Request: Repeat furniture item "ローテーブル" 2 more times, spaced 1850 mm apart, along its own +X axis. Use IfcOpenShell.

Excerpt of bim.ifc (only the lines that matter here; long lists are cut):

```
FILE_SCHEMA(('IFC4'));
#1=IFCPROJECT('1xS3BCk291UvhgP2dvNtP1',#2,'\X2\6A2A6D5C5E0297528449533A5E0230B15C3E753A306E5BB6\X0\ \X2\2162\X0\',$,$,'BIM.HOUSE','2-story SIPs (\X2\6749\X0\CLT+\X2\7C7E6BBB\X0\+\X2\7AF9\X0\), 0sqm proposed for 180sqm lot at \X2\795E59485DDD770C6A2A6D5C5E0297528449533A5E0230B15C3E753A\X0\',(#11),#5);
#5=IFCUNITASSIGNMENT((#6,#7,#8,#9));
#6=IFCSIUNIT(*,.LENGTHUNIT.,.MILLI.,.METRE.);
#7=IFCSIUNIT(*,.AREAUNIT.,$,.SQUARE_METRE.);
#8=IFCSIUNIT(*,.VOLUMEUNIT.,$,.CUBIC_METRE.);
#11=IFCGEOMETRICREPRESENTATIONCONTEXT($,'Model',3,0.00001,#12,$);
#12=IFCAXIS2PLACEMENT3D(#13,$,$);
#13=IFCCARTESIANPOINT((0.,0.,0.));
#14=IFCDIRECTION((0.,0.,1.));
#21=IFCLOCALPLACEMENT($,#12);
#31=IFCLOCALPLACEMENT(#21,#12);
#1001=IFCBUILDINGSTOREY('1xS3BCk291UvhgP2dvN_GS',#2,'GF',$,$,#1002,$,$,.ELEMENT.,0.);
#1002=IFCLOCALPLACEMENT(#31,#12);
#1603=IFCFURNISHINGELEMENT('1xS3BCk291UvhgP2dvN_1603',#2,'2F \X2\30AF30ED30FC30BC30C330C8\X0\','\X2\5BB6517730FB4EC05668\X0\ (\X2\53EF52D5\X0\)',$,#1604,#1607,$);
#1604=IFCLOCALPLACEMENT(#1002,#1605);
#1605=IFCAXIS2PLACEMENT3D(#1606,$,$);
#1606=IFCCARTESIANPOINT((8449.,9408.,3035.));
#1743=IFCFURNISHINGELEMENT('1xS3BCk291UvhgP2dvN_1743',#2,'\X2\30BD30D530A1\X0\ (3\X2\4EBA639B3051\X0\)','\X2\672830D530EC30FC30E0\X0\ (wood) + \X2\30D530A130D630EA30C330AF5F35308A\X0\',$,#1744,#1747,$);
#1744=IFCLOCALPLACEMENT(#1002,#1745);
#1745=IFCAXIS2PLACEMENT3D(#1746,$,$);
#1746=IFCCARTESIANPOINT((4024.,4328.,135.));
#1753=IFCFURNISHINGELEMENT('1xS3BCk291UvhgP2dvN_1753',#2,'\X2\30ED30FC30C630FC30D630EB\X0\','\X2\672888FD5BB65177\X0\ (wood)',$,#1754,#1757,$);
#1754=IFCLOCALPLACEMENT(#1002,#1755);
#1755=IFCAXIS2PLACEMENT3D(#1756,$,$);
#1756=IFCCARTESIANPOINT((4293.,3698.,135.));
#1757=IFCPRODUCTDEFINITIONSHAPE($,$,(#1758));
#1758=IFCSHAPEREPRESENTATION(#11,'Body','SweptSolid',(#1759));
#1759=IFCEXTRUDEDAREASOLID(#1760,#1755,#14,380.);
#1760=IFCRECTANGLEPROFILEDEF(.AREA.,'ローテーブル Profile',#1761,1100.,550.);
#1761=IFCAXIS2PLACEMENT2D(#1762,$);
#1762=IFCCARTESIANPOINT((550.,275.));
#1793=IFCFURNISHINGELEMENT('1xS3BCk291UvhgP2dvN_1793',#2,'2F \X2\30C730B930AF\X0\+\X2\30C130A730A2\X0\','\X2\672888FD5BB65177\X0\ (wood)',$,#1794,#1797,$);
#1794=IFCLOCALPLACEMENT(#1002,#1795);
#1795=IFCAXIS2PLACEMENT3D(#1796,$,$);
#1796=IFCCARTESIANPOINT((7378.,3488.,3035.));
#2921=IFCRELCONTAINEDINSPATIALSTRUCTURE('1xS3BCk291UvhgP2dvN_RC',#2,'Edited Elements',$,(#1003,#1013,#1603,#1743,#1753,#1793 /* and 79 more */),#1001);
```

```python
import ifcopenshell
import ifcopenshell.api.geometry
import ifcopenshell.api.root
import ifcopenshell.util.element
import ifcopenshell.util.placement
import ifcopenshell.util.unit

model = ifcopenshell.open("bim.ifc")
unit_scale = ifcopenshell.util.unit.calculate_unit_scale(model)


def reuse_history(source, copy):
    """copy_class also copies each property set's owner history, people and application; keep the originals."""
    for rel in copy.IsDefinedBy:
        if rel.is_a("IfcRelDefinesByProperties") and (history := rel.RelatingPropertyDefinition.OwnerHistory):
            rel.RelatingPropertyDefinition.OwnerHistory = source.OwnerHistory
            ifcopenshell.util.element.remove_deep2(model, history)


source = model.by_guid("1xS3BCk291UvhgP2dvN_1753")
base = ifcopenshell.util.placement.get_local_placement(source.ObjectPlacement)
step = base[:3, 0] * 1.85 / unit_scale

for i in range(1, 3):
    copy = ifcopenshell.api.root.copy_class(model, product=source)
    copy.Representation = ifcopenshell.util.element.copy_deep(
        model, source.Representation, exclude=["IfcGeometricRepresentationContext", "IfcRepresentationMap"]
    )
    reuse_history(source, copy)
    matrix = base.copy()
    matrix[:3, 3] += i * step
    print("added at", matrix[:3, 3].round(3) + 0.0)
    ifcopenshell.api.geometry.edit_object_placement(model, product=copy, matrix=matrix, is_si=False)

model.write("bim_updated.ifc")
```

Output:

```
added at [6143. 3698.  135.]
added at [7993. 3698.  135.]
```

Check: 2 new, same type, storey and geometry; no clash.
